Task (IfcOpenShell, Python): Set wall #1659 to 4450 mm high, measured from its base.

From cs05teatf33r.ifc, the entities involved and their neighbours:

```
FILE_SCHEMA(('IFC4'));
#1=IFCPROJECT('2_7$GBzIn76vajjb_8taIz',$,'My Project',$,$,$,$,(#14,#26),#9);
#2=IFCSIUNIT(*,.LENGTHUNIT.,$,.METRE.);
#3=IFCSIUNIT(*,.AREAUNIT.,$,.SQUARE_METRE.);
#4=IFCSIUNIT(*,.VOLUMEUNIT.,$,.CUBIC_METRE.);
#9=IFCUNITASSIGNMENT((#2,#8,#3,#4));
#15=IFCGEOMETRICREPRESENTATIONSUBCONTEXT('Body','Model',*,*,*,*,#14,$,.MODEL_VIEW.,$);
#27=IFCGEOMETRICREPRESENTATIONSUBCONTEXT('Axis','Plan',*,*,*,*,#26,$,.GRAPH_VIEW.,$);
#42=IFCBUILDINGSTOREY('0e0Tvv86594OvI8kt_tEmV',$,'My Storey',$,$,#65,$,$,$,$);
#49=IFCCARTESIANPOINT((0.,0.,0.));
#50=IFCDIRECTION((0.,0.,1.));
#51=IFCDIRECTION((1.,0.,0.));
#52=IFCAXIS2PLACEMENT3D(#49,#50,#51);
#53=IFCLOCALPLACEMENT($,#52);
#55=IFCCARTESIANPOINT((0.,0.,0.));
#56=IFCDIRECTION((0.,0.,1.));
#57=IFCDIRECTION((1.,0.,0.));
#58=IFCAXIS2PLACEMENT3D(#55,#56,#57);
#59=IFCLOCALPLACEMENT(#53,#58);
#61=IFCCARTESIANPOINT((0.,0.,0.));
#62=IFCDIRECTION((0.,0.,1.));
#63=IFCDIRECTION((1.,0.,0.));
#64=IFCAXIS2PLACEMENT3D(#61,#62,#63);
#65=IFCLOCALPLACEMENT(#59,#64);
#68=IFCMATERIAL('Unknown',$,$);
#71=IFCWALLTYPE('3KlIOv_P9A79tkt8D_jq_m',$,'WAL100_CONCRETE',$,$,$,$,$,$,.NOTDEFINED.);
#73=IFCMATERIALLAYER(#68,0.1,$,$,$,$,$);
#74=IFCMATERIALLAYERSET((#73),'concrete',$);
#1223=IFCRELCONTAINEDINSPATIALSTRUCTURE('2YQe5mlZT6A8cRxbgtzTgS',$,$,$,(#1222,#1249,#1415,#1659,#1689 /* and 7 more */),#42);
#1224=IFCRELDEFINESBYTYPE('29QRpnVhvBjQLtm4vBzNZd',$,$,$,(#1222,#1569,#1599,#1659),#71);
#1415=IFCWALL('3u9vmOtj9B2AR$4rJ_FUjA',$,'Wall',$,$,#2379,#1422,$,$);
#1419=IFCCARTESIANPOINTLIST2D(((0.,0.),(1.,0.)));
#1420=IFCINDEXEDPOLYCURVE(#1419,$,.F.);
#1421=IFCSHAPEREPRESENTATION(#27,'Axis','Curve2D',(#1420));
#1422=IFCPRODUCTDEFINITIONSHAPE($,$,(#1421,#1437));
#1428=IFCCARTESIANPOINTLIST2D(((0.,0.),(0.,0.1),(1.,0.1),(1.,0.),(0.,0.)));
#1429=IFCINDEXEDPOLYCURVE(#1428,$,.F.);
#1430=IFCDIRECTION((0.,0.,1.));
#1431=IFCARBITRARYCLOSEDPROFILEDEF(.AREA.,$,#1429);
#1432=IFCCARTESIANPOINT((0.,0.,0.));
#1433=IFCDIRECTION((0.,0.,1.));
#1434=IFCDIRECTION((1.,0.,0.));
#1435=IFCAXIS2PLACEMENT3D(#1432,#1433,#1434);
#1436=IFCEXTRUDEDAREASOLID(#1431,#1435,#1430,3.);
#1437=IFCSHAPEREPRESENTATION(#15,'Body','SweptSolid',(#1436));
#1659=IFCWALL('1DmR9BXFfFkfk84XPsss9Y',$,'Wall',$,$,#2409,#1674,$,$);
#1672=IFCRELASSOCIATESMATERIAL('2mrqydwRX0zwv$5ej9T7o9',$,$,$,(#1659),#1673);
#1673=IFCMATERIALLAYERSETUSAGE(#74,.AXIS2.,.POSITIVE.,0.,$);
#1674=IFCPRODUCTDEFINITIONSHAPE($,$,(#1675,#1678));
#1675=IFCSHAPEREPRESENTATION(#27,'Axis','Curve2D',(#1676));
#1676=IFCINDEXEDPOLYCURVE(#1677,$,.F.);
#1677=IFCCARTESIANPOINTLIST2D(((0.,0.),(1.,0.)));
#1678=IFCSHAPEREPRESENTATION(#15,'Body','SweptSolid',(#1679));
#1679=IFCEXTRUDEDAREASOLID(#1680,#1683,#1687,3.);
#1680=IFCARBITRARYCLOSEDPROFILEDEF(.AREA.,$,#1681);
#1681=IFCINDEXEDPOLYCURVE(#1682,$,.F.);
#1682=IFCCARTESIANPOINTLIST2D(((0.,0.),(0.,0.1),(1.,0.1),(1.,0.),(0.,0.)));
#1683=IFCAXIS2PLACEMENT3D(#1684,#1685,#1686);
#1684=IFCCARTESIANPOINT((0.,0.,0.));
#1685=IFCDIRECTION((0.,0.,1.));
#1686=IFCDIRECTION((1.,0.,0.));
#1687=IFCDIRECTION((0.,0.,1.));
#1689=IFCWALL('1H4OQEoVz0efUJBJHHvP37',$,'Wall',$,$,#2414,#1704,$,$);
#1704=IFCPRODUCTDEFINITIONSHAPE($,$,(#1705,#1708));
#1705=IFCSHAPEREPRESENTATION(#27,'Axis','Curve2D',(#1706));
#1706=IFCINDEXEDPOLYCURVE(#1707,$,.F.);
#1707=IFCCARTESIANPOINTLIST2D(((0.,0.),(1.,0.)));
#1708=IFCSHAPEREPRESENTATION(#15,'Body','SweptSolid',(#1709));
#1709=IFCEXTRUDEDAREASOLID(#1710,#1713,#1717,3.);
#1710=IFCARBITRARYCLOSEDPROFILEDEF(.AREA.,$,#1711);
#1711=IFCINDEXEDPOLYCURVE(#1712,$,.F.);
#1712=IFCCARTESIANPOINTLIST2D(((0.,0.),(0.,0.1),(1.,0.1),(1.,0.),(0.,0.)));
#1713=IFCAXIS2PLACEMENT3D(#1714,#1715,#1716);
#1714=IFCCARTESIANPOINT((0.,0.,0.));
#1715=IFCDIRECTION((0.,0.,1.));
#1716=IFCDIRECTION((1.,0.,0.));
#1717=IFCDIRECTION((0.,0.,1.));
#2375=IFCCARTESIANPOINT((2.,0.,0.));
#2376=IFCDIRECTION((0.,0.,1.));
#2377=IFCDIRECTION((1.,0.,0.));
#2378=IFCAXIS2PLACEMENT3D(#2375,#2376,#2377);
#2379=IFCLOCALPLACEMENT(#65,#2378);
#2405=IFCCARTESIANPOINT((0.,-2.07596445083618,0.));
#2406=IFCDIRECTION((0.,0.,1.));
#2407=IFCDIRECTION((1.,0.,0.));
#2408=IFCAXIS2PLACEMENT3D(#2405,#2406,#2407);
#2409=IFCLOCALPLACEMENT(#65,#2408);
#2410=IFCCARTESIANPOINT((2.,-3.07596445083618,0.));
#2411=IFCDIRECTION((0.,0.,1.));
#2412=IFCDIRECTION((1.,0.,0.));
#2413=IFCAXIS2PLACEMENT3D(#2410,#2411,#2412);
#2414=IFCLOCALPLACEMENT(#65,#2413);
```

```python
import ifcopenshell
import ifcopenshell.geom
import ifcopenshell.util.representation
import ifcopenshell.util.shape
import ifcopenshell.util.unit

model = ifcopenshell.open("cs05teatf33r.ifc")
unit_scale = ifcopenshell.util.unit.calculate_unit_scale(model)
settings = ifcopenshell.geom.settings()


def volume(element):
    """Net volume in cubic metres, openings subtracted."""
    shape = ifcopenshell.geom.create_shape(settings, element)
    return ifcopenshell.util.shape.get_volume(shape.geometry)


wall = model.by_guid("1DmR9BXFfFkfk84XPsss9Y")
before = volume(wall)

body = ifcopenshell.util.representation.get_representation(wall, "Model", "Body")
solid = body.Items[0]
old_height = solid.Depth
solid.Depth = 4.45 / unit_scale
after = volume(wall)

print(f"height {old_height:g} -> {solid.Depth:g}, volume {before:.3f} -> {after:.3f} m3")

model.write("cs05teatf33r-out.ifc")
```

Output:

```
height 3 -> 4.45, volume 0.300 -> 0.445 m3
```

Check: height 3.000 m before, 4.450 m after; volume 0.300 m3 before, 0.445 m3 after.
